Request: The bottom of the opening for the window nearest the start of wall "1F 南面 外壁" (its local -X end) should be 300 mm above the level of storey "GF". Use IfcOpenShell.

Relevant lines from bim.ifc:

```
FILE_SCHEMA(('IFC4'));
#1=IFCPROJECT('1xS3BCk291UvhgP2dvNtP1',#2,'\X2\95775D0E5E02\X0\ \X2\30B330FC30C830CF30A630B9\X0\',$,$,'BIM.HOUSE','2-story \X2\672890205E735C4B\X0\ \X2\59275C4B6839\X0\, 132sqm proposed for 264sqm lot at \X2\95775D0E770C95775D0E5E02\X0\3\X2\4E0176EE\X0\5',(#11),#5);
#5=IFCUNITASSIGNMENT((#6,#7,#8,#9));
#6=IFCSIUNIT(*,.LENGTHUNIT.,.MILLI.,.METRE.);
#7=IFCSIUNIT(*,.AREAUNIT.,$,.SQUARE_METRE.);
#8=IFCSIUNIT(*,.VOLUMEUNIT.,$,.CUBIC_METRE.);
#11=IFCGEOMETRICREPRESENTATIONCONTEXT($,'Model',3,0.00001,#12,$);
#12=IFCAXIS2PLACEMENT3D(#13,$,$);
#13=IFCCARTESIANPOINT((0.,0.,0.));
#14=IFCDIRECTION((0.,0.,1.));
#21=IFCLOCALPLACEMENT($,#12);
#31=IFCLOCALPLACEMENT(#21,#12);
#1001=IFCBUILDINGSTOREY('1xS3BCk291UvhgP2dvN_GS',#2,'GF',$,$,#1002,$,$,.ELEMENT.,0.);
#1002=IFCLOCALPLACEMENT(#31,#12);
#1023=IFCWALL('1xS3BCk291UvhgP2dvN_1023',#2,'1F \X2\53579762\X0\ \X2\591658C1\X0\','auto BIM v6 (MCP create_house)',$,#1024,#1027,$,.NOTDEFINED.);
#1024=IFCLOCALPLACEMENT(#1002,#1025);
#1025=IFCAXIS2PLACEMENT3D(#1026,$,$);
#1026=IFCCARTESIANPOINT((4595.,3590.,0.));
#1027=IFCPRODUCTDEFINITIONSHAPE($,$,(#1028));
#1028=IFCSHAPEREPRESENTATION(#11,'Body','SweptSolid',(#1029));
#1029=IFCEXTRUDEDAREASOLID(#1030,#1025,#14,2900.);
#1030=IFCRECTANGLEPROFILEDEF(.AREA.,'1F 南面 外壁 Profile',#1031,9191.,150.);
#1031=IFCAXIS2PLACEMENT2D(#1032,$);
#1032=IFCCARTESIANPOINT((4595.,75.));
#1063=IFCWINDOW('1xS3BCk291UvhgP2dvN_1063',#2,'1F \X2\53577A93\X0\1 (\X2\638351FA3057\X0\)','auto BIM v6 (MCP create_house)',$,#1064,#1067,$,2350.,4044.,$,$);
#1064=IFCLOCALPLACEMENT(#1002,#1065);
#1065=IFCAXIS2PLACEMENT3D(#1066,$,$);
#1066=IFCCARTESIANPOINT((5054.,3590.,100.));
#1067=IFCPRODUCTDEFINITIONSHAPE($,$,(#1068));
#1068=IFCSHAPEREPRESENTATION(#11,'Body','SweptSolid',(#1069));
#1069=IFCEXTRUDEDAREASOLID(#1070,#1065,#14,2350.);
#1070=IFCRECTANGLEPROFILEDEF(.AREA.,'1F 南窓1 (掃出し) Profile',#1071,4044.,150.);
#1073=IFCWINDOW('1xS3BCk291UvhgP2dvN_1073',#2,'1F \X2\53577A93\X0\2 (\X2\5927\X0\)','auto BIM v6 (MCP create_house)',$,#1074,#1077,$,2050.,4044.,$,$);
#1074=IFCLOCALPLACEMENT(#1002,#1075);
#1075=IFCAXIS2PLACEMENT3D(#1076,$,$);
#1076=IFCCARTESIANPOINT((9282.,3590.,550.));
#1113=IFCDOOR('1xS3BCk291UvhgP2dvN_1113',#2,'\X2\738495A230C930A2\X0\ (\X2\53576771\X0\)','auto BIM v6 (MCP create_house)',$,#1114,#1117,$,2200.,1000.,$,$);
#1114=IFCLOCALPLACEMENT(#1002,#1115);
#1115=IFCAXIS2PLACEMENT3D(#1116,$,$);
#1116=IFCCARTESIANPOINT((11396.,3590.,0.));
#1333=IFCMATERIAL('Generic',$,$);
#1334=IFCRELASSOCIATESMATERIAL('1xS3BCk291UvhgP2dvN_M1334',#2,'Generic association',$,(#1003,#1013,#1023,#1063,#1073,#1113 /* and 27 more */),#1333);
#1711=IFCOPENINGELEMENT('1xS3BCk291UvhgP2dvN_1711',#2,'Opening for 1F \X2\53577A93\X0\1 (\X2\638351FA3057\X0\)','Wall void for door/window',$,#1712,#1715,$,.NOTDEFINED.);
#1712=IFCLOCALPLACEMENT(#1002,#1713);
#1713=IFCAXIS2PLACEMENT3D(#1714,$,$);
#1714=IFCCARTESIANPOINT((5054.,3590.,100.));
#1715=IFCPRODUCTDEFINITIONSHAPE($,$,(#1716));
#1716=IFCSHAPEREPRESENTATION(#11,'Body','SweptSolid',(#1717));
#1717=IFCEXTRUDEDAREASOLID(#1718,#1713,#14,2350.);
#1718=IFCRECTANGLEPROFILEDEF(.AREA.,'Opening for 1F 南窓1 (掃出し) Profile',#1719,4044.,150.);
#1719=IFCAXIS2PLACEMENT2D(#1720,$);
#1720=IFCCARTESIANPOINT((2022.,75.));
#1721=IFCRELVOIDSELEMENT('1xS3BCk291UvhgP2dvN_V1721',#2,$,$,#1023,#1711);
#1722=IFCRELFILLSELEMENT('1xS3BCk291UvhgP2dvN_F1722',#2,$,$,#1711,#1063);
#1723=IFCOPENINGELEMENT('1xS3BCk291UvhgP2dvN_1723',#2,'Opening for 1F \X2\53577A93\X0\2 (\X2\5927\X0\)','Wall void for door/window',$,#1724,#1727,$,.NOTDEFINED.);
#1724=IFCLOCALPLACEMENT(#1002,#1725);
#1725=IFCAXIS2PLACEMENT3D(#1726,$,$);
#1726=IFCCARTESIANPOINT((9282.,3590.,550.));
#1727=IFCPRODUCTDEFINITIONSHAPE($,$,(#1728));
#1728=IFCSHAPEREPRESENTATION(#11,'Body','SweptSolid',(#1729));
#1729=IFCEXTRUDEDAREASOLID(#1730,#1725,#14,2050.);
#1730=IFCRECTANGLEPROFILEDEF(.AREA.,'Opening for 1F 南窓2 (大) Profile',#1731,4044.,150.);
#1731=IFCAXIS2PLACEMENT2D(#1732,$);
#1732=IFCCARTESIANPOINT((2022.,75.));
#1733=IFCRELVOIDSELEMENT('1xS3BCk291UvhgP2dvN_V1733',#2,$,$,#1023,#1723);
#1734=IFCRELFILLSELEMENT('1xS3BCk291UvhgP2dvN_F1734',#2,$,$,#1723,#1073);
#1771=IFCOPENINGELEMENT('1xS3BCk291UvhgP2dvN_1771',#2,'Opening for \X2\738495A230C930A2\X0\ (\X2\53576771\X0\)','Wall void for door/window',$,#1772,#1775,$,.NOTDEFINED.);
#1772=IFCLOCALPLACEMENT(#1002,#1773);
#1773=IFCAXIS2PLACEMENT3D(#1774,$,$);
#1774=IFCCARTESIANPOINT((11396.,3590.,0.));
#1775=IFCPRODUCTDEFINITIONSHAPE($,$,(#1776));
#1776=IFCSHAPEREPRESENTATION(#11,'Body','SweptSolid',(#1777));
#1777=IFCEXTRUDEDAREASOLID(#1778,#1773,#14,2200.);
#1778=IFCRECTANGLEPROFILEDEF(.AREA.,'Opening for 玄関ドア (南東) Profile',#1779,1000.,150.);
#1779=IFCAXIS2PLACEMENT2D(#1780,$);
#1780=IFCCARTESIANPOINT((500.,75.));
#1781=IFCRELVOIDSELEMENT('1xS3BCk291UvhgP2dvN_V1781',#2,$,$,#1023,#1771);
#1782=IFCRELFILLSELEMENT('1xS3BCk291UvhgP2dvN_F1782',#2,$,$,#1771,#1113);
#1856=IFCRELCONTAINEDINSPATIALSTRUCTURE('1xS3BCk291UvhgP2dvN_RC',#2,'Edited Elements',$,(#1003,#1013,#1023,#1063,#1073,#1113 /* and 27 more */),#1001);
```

```python
import numpy as np
import ifcopenshell
import ifcopenshell.api.geometry
import ifcopenshell.geom
import ifcopenshell.util.element
import ifcopenshell.util.placement
import ifcopenshell.util.shape
import ifcopenshell.util.unit

model = ifcopenshell.open("bim.ifc")
unit_scale = ifcopenshell.util.unit.calculate_unit_scale(model)

window = model.by_id(1063)
opening = window.FillsVoids[0].RelatingOpeningElement
storey = ifcopenshell.util.element.get_container(window, ifc_class="IfcBuildingStorey")
level = ifcopenshell.util.placement.get_local_placement(storey.ObjectPlacement)[2, 3]

# The opening's origin need not be at the sill, so measure its lowest point.
shape = ifcopenshell.geom.create_shape(ifcopenshell.geom.settings(), opening)
bottom = ifcopenshell.util.shape.get_shape_bottom_elevation(shape, shape.geometry) / unit_scale
dz = level + 0.3 / unit_scale - bottom

shift = np.array([0.0, 0.0, dz])
# The window is not placed relative to its opening, so move both.
for product in (opening, window):
    matrix = ifcopenshell.util.placement.get_local_placement(product.ObjectPlacement)
    matrix[:3, 3] += shift
    ifcopenshell.api.geometry.edit_object_placement(model, product=product, matrix=matrix, is_si=False)

print(f"moved by {dz * unit_scale:+.3f} m")

model.write("bim_edited.ifc")
```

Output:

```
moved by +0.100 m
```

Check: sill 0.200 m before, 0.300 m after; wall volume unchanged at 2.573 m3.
